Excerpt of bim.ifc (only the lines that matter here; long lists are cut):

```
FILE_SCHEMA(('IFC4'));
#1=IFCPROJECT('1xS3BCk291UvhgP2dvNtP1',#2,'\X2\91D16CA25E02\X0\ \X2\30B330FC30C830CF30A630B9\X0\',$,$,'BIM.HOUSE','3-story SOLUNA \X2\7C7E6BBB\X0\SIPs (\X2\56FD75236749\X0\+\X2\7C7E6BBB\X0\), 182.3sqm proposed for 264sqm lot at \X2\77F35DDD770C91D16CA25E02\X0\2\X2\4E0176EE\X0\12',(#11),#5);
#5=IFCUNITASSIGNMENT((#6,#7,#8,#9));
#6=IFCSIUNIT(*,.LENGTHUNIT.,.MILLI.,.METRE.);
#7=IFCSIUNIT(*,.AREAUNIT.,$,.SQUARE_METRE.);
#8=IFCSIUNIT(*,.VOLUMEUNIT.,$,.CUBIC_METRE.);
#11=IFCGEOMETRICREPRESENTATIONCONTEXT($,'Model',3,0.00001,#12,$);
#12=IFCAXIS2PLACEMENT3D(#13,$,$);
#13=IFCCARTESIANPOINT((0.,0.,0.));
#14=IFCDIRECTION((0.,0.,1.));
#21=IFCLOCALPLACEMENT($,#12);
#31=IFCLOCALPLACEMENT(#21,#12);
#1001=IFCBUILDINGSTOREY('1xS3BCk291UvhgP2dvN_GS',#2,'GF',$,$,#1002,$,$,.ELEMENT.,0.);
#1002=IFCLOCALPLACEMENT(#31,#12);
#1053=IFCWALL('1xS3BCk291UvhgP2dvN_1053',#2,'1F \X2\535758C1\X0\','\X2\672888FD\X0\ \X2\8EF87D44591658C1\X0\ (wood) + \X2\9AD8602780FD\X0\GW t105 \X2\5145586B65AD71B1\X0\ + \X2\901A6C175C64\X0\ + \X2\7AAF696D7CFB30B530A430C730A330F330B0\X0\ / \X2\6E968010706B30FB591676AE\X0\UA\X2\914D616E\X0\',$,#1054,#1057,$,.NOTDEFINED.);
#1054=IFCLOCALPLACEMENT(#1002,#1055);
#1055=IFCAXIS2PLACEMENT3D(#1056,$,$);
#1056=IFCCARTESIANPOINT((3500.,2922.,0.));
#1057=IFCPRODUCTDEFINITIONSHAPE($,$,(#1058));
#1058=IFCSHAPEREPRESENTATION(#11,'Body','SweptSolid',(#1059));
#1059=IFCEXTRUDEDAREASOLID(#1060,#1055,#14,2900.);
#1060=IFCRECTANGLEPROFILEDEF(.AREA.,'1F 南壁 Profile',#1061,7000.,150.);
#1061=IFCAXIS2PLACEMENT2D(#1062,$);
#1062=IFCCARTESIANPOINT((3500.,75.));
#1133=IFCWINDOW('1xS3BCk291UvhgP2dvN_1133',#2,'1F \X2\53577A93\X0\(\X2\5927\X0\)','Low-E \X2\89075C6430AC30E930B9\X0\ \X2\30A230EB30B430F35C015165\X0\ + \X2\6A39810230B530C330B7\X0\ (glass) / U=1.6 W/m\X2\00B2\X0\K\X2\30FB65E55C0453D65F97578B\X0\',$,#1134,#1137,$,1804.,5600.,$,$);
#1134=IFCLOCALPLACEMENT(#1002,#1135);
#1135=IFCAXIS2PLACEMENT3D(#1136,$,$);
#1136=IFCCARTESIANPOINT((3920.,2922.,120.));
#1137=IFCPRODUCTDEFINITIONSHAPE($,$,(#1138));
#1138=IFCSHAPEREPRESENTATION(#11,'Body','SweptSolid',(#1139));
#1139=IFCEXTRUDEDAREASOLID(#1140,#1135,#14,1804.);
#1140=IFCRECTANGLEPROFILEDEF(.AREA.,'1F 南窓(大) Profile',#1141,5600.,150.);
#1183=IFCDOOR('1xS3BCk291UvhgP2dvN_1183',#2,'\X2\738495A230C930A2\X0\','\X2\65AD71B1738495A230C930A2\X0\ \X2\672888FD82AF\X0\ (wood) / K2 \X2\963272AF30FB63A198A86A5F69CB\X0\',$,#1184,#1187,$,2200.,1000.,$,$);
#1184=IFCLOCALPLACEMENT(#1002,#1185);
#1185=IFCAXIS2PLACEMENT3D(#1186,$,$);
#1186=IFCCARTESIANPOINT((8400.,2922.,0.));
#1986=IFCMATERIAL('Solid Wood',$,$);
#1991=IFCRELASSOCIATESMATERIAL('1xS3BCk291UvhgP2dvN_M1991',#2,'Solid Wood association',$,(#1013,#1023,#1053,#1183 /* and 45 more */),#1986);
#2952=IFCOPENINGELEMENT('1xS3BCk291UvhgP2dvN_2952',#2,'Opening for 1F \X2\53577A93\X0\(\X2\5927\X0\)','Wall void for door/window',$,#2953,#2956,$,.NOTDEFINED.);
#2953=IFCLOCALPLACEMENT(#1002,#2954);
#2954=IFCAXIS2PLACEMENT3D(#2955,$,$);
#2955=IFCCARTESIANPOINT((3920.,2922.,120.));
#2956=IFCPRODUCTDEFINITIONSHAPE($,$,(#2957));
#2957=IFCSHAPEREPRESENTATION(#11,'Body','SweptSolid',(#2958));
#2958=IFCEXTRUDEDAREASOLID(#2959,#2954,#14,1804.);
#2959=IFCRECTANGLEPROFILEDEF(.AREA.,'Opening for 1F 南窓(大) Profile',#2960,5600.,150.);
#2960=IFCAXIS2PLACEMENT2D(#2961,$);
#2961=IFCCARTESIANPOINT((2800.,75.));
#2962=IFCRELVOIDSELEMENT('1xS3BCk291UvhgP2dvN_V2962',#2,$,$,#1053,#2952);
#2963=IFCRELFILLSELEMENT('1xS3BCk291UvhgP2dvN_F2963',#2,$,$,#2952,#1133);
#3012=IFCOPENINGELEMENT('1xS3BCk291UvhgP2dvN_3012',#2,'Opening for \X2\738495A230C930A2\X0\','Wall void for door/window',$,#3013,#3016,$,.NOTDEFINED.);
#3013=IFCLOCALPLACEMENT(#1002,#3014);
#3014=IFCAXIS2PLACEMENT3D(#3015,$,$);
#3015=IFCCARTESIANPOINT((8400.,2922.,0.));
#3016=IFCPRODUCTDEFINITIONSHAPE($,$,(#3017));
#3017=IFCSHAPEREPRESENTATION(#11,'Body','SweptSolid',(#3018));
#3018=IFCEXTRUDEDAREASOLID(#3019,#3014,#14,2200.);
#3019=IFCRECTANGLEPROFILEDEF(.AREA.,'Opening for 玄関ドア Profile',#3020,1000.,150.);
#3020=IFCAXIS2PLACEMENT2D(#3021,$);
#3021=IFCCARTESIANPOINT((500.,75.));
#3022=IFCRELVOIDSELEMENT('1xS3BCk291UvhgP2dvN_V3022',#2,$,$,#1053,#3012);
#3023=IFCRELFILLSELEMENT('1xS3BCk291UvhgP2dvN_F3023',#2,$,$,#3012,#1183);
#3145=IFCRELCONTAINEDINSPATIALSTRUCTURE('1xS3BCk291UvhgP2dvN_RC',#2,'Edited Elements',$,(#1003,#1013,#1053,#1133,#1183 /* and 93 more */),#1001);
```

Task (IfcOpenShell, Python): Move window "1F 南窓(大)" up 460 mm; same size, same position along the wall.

```python
import numpy as np
import ifcopenshell
import ifcopenshell.api.geometry
import ifcopenshell.util.placement
import ifcopenshell.util.unit

model = ifcopenshell.open("bim.ifc")
unit_scale = ifcopenshell.util.unit.calculate_unit_scale(model)

window = model.by_guid("1xS3BCk291UvhgP2dvN_1133")
opening = window.FillsVoids[0].RelatingOpeningElement
dz = 460.0

shift = np.array([0.0, 0.0, dz])
# The window is not placed relative to its opening, so move both.
for product in (opening, window):
    matrix = ifcopenshell.util.placement.get_local_placement(product.ObjectPlacement)
    matrix[:3, 3] += shift
    ifcopenshell.api.geometry.edit_object_placement(model, product=product, matrix=matrix, is_si=False)

print(f"moved by {dz * unit_scale:+.3f} m")

model.write("bim_edited.ifc")
```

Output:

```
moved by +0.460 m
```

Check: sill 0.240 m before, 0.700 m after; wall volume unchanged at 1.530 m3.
